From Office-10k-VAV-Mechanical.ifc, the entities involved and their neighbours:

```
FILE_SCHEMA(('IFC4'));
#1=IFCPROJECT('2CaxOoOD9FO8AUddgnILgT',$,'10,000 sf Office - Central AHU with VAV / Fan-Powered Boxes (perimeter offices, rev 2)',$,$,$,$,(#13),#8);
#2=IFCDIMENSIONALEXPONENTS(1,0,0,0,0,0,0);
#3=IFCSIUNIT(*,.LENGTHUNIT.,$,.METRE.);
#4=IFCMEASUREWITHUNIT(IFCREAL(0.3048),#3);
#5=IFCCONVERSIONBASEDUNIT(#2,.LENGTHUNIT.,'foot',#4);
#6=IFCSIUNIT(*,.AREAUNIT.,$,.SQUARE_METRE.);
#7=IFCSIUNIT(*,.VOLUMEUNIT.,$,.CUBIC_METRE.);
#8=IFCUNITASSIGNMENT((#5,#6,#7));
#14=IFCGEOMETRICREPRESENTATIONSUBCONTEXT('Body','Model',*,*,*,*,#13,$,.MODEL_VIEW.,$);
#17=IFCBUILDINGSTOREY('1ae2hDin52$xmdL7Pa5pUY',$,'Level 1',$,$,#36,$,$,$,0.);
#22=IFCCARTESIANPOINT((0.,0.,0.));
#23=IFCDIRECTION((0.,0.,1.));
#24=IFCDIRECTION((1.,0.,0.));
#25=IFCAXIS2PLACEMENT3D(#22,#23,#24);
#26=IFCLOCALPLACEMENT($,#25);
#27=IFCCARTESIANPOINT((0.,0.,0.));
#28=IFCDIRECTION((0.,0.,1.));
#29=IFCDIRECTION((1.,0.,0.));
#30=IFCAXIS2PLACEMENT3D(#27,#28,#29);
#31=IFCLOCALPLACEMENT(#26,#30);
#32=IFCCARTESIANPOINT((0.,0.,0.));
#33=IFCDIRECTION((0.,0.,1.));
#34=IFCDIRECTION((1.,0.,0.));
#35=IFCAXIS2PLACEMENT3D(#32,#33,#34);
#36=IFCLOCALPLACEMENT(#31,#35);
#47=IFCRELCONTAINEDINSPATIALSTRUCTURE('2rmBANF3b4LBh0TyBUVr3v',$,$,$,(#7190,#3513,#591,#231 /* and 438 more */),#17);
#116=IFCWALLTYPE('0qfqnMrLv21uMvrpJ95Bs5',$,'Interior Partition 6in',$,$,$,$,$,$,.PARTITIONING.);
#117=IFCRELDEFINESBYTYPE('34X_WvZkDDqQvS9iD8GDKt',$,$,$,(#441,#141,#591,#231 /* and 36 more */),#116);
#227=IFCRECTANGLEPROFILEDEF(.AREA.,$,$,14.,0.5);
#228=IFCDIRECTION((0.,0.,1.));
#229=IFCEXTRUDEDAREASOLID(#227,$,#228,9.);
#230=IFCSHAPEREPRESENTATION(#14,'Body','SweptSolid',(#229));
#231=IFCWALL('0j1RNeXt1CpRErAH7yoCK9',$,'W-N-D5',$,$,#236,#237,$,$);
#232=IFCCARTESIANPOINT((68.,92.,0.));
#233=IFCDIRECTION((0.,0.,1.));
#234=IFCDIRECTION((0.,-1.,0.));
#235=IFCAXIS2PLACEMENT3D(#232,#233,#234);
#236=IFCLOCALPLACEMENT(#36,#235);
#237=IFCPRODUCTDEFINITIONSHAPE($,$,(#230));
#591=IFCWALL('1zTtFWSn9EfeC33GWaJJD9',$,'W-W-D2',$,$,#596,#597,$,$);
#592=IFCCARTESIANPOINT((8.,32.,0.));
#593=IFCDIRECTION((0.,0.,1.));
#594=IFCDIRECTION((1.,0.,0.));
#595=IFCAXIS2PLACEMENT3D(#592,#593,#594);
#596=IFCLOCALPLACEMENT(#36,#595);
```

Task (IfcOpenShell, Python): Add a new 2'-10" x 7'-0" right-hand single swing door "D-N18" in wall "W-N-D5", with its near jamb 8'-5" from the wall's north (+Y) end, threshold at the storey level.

```python
import numpy as np
import ifcopenshell
import ifcopenshell.api.feature
import ifcopenshell.api.geometry
import ifcopenshell.api.root
import ifcopenshell.api.spatial
import ifcopenshell.geom
import ifcopenshell.util.element
import ifcopenshell.util.placement
import ifcopenshell.util.representation
import ifcopenshell.util.shape
import ifcopenshell.util.unit

model = ifcopenshell.open("Office-10k-VAV-Mechanical.ifc")
unit_scale = ifcopenshell.util.unit.calculate_unit_scale(model)
settings = ifcopenshell.geom.settings()


def volume(element):
    """Net volume in cubic metres, openings subtracted."""
    shape = ifcopenshell.geom.create_shape(settings, element)
    return ifcopenshell.util.shape.get_volume(shape.geometry)


wall = model.by_guid("0j1RNeXt1CpRErAH7yoCK9")
storey = ifcopenshell.util.element.get_container(wall, ifc_class="IfcBuildingStorey")
context = ifcopenshell.util.representation.get_context(model, "Model", "Body", "MODEL_VIEW")
before = volume(wall)

width, height, from_end, sill = 0.8636, 2.1336, 2.5654, 0.0  # metres

# The wall runs along its own X axis, and the end named is its -X end.
wall_shape = ifcopenshell.geom.create_shape(settings, wall)
x, y, z = ifcopenshell.util.shape.get_vertices(wall_shape.geometry).T
start = x.min() + from_end
face, thickness = float(y.min()), float(y.max() - y.min())
wall_matrix = ifcopenshell.util.placement.get_local_placement(wall.ObjectPlacement)
level = ifcopenshell.util.placement.get_local_placement(storey.ObjectPlacement)[2, 3]


def in_wall(x, y):
    """Placement at x, y metres in the wall's axes, at sill height."""
    matrix = wall_matrix.copy()
    matrix[:, 3] = wall_matrix @ np.array([x / unit_scale, y / unit_scale, 0.0, 1.0])
    matrix[2, 3] = level + sill / unit_scale
    return matrix


# Opening: a box that overshoots both wall faces by 50 mm.
opening = ifcopenshell.api.root.create_entity(model, ifc_class="IfcOpeningElement", predefined_type="OPENING")
box = ifcopenshell.api.geometry.add_wall_representation(
    model, context=context, length=width, height=height, thickness=thickness + 0.1
)
ifcopenshell.api.geometry.assign_representation(model, product=opening, representation=box)
ifcopenshell.api.geometry.edit_object_placement(model, product=opening, matrix=in_wall(start, face - 0.05), is_si=False)
ifcopenshell.api.feature.add_feature(model, feature=opening, element=wall)

door = ifcopenshell.api.root.create_entity(model, ifc_class="IfcDoor", name="D-N18", predefined_type="DOOR")
door.OverallWidth, door.OverallHeight = width / unit_scale, height / unit_scale
door.OperationType = "SINGLE_SWING_RIGHT"
body = ifcopenshell.api.geometry.add_door_representation(
    model,
    context=context,
    overall_width=door.OverallWidth,
    overall_height=door.OverallHeight,
    operation_type="SINGLE_SWING_RIGHT",
    lining_properties={"LiningDepth": thickness / unit_scale, "ThresholdDepth": thickness / unit_scale},
)
ifcopenshell.api.geometry.assign_representation(model, product=door, representation=body)
ifcopenshell.api.spatial.assign_container(model, products=[door], relating_structure=storey)
ifcopenshell.api.feature.add_filling(model, opening=opening, element=door)

# The lining spans the wall, so the door starts at the wall face.
ifcopenshell.api.geometry.edit_object_placement(model, product=door, matrix=in_wall(start, face), is_si=False)

after = volume(wall)

print(f"wall volume {before:.3f} -> {after:.3f} m3")

model.write("Office-10k-VAV-Mechanical-out.ifc")
```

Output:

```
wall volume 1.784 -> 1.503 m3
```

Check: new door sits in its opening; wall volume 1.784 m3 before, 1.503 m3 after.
